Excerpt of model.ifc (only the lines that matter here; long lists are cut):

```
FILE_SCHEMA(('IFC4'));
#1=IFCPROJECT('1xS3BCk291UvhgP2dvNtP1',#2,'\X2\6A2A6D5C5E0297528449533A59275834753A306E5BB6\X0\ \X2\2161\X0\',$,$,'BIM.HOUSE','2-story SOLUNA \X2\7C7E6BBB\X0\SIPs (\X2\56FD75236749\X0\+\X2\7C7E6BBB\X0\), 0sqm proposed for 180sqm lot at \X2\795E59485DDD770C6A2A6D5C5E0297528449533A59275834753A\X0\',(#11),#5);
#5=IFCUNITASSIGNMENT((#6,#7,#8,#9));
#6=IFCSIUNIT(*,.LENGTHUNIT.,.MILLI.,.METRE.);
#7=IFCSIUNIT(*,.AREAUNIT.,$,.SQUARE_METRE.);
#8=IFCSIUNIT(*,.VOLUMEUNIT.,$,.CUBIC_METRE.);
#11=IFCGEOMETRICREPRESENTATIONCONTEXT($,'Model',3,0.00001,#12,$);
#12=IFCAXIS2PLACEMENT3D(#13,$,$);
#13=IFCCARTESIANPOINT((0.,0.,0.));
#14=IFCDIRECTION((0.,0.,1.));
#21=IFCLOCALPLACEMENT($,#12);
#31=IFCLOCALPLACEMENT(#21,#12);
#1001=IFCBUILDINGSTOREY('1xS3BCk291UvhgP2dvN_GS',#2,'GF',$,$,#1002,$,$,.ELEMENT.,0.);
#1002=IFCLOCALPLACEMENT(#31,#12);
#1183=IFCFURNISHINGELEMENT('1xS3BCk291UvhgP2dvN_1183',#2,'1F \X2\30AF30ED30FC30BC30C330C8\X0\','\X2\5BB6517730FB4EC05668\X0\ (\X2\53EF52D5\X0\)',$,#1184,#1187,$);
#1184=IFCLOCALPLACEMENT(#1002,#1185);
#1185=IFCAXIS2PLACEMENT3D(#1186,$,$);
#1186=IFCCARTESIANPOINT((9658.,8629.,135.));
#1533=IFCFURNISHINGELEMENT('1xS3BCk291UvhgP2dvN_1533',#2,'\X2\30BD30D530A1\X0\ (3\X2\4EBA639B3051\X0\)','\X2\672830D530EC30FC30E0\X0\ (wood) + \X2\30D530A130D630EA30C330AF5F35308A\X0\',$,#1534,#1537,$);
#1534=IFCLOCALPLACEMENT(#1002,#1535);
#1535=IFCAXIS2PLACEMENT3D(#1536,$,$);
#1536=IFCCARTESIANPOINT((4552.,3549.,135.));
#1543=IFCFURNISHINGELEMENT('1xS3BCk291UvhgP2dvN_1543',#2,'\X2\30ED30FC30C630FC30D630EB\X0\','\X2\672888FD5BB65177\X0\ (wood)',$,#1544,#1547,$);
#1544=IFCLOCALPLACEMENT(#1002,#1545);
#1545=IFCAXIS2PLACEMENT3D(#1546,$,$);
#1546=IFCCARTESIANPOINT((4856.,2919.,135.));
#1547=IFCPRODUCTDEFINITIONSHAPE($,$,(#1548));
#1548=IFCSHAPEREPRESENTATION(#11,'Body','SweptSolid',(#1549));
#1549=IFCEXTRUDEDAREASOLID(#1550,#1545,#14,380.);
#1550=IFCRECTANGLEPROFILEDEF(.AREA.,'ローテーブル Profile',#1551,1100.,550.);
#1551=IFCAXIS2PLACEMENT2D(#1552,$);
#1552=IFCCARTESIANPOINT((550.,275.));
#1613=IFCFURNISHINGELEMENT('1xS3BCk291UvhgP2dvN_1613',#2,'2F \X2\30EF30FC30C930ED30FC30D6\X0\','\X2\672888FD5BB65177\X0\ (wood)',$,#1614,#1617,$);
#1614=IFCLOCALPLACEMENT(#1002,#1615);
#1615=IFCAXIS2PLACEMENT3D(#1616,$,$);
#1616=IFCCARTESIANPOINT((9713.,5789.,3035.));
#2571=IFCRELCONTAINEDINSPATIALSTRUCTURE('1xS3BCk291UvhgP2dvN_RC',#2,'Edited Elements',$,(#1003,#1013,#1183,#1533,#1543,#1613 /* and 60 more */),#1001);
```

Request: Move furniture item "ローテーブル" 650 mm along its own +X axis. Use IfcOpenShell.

```python
import ifcopenshell
import ifcopenshell.api.geometry
import ifcopenshell.util.placement

model = ifcopenshell.open("model.ifc")

item = model.by_guid("1xS3BCk291UvhgP2dvN_1543")
matrix = ifcopenshell.util.placement.get_local_placement(item.ObjectPlacement)
matrix[:3, 3] += matrix[:3, 0] * 650.0
ifcopenshell.api.geometry.edit_object_placement(model, product=item, matrix=matrix, is_si=False)

print(ifcopenshell.util.placement.get_local_placement(item.ObjectPlacement).round(3) + 0.0)

model.write("model-out.ifc")
```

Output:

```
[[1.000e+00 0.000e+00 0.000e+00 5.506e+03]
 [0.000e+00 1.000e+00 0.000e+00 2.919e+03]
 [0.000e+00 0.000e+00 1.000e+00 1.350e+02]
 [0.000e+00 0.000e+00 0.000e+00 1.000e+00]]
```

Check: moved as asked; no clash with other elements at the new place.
